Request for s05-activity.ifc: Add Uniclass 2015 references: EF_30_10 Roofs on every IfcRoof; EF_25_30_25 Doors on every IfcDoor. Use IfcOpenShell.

First a look at what the model holds.

```python
import ifcopenshell

model = ifcopenshell.open("s05-activity.ifc")
print(model.schema)
print("classifications:", [c.Name for c in model.by_type("IfcClassification")])
for ifc_class in ("IfcDoor", "IfcRoof", "IfcStair", "IfcWall", "IfcWindow"):
    print(ifc_class, len(model.by_type(ifc_class)))
```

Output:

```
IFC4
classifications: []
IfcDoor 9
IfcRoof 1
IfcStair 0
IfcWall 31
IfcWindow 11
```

```python
import ifcopenshell
import ifcopenshell.api.classification

model = ifcopenshell.open("s05-activity.ifc")

system = ifcopenshell.api.classification.add_classification(model, classification="Uniclass 2015")

codes = {
    "IfcRoof": ("EF_30_10", "Roofs"),
    "IfcDoor": ("EF_25_30_25", "Doors"),
}
for ifc_class, (code, name) in codes.items():
    products = model.by_type(ifc_class)
    ifcopenshell.api.classification.add_reference(
        model, products=products, classification=system, identification=code, name=name
    )
    print(code, len(products))

model.write("s05-activity_v2.ifc")
```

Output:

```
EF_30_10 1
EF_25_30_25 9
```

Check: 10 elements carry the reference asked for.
